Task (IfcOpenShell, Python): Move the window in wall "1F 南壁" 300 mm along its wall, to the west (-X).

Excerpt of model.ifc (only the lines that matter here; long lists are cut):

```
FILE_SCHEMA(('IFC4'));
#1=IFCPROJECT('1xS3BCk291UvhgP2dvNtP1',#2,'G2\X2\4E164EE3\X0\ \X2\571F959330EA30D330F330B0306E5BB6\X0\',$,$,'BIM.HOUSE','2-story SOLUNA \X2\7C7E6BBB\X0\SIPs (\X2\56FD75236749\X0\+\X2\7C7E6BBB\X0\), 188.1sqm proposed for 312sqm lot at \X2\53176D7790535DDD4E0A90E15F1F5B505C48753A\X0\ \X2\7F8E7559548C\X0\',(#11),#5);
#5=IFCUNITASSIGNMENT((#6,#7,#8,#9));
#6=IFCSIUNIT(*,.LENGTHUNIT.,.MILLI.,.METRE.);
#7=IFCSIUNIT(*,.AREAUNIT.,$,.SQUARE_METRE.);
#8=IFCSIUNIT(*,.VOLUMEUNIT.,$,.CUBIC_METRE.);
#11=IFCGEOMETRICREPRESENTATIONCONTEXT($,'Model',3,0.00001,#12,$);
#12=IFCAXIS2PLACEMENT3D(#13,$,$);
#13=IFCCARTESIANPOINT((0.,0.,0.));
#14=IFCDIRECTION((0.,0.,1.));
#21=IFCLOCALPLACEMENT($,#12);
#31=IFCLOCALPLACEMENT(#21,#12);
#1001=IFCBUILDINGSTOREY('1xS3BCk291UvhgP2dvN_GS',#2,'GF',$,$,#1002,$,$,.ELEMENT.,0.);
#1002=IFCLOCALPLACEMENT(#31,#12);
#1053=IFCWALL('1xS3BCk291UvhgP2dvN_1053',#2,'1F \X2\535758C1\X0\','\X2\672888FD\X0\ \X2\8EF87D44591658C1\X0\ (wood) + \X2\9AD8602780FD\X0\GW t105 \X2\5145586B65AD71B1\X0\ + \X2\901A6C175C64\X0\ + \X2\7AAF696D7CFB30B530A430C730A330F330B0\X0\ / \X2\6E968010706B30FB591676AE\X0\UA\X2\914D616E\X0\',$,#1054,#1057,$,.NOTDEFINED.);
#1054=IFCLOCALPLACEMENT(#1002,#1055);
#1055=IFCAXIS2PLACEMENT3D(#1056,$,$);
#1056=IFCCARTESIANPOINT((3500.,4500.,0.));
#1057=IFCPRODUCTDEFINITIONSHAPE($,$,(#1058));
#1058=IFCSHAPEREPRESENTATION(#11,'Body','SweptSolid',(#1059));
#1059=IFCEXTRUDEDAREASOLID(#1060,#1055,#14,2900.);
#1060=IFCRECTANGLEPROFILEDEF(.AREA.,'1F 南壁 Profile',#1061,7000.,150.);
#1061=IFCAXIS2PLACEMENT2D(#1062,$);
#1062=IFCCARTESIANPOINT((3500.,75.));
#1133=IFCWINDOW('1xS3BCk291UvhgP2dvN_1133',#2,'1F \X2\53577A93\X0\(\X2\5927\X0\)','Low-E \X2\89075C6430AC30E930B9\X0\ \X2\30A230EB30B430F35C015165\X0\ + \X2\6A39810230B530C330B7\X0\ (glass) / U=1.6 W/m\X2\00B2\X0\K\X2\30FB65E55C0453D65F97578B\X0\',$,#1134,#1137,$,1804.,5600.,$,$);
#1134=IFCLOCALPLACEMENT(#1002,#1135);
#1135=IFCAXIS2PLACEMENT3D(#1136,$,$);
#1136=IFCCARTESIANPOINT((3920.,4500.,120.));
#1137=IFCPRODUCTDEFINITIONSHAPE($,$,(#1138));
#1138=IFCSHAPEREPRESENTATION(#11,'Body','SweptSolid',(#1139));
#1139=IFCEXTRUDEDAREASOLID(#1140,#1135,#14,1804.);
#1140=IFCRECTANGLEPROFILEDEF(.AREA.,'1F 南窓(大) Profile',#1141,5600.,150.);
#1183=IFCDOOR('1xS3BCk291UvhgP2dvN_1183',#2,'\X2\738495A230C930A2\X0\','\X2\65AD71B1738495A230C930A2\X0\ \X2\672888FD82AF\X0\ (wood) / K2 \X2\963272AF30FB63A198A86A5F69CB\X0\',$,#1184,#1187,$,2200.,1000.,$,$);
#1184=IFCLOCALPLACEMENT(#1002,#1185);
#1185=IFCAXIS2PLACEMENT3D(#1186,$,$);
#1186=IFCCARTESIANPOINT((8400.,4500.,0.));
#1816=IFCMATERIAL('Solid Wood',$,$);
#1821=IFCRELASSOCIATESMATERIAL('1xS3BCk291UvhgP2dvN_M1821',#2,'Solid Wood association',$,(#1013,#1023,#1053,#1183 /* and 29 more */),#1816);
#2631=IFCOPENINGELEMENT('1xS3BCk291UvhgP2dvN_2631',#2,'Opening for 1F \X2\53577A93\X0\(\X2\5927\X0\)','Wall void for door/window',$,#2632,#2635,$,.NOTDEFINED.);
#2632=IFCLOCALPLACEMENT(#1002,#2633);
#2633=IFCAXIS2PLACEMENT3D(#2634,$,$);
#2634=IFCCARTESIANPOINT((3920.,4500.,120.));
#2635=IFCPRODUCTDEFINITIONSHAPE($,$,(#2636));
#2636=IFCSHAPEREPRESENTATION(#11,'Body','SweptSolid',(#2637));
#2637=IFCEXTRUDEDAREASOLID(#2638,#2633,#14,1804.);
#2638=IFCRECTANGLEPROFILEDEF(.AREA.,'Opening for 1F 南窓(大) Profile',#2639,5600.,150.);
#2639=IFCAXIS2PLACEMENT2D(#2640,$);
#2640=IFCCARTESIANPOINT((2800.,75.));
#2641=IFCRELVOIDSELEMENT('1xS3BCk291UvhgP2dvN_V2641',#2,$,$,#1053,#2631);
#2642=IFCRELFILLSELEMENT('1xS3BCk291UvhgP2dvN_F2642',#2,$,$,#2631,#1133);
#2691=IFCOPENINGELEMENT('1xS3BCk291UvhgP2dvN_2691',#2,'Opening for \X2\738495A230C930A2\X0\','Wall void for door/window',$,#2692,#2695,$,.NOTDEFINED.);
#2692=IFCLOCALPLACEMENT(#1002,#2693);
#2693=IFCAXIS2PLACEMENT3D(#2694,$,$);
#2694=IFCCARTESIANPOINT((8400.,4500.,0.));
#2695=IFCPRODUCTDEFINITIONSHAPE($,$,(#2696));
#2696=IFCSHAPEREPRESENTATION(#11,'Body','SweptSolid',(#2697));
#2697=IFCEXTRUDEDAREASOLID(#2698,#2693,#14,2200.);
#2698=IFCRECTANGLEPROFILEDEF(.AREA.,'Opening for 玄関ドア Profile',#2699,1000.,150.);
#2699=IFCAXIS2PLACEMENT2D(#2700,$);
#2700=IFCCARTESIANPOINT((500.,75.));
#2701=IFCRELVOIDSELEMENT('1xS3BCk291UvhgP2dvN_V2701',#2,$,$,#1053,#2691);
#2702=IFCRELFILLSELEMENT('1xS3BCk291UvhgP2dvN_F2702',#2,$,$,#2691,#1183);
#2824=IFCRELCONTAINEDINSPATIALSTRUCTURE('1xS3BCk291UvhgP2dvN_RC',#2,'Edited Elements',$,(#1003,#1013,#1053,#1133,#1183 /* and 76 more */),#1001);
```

```python
import ifcopenshell
import ifcopenshell.api.geometry
import ifcopenshell.util.placement
import ifcopenshell.util.unit

model = ifcopenshell.open("model.ifc")
unit_scale = ifcopenshell.util.unit.calculate_unit_scale(model)

window = model.by_guid("1xS3BCk291UvhgP2dvN_1133")
opening = window.FillsVoids[0].RelatingOpeningElement
wall = opening.VoidsElements[0].RelatingBuildingElement

wall_matrix = ifcopenshell.util.placement.get_local_placement(wall.ObjectPlacement)
shift = wall_matrix[:3, 0] * -0.3 / unit_scale
before = ifcopenshell.util.placement.get_local_placement(window.ObjectPlacement)[:3, 3].copy()

# The window is not placed relative to its opening, so move both.
for product in (opening, window):
    matrix = ifcopenshell.util.placement.get_local_placement(product.ObjectPlacement)
    matrix[:3, 3] += shift
    ifcopenshell.api.geometry.edit_object_placement(model, product=product, matrix=matrix, is_si=False)

after = ifcopenshell.util.placement.get_local_placement(window.ObjectPlacement)[:3, 3]
print("window moved by", (after - before).round(3) + 0.0)

model.write("model_rev.ifc")
```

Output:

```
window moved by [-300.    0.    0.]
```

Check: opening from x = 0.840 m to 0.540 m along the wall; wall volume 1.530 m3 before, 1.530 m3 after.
